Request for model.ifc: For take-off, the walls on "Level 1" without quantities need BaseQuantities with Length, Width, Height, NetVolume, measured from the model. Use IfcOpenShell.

First a look at what the model holds.

```python
import ifcopenshell
import ifcopenshell.util.element
import ifcopenshell.util.unit

model = ifcopenshell.open("model.ifc")
print(model.schema)
for unit_type in ("LENGTHUNIT", "AREAUNIT", "VOLUMEUNIT"):
    print(unit_type, ifcopenshell.util.unit.calculate_unit_scale(model, unit_type))
storey = next(s for s in model.by_type("IfcBuildingStorey") if s.Name == "Level 1")
walls = [e for e in ifcopenshell.util.element.get_decomposition(storey) if e.is_a("IfcWall")]
for e in sorted(walls, key=lambda e: e.id()):
    print(e.id(), e.is_a(), e.Name, list(ifcopenshell.util.element.get_psets(e, qtos_only=True)), sep=" | ")
```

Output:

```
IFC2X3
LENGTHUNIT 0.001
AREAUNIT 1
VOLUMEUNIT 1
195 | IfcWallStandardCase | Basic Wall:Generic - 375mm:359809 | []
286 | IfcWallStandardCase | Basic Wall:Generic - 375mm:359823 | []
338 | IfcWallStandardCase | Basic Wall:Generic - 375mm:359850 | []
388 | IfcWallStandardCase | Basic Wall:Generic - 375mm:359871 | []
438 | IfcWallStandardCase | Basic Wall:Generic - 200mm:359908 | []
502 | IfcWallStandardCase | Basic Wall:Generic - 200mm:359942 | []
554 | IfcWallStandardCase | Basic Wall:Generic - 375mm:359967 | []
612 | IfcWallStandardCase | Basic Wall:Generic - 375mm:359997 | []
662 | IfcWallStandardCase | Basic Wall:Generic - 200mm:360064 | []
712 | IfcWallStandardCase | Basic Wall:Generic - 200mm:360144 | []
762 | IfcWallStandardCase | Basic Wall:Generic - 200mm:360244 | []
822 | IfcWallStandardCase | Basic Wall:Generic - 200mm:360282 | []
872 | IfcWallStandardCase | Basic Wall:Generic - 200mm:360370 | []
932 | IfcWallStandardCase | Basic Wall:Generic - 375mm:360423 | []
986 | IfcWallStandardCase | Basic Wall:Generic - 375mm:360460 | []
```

```python
import ifcopenshell
import ifcopenshell.api.pset
import ifcopenshell.geom
import ifcopenshell.util.element
import ifcopenshell.util.shape
import ifcopenshell.util.unit

model = ifcopenshell.open("model.ifc")
unit_scale = ifcopenshell.util.unit.calculate_unit_scale(model)
volume_scale = ifcopenshell.util.unit.calculate_unit_scale(model, "VOLUMEUNIT")
settings = ifcopenshell.geom.settings()

storey = next(s for s in model.by_type("IfcBuildingStorey") if s.Name == "Level 1")
walls = [e for e in ifcopenshell.util.element.get_decomposition(storey) if e.is_a("IfcWall")]

for e in sorted(walls, key=lambda e: e.id()):
    if ifcopenshell.util.element.get_psets(e, qtos_only=True, should_inherit=False):
        continue
    # Geometry comes back in metres, in the element's own axes.
    shape = ifcopenshell.geom.create_shape(settings, e)
    values = {
        "Length": ifcopenshell.util.shape.get_x(shape.geometry) / unit_scale,
        "Width": ifcopenshell.util.shape.get_y(shape.geometry) / unit_scale,
        "Height": ifcopenshell.util.shape.get_z(shape.geometry) / unit_scale,
        "NetVolume": ifcopenshell.util.shape.get_volume(shape.geometry) / volume_scale,
    }
    qto = ifcopenshell.api.pset.add_qto(model, product=e, name="BaseQuantities")
    ifcopenshell.api.pset.edit_qto(model, qto=qto, properties=values)
    print(e.id(), {k: round(v, 3) for k, v in values.items()})

model.write("model_rev.ifc")
```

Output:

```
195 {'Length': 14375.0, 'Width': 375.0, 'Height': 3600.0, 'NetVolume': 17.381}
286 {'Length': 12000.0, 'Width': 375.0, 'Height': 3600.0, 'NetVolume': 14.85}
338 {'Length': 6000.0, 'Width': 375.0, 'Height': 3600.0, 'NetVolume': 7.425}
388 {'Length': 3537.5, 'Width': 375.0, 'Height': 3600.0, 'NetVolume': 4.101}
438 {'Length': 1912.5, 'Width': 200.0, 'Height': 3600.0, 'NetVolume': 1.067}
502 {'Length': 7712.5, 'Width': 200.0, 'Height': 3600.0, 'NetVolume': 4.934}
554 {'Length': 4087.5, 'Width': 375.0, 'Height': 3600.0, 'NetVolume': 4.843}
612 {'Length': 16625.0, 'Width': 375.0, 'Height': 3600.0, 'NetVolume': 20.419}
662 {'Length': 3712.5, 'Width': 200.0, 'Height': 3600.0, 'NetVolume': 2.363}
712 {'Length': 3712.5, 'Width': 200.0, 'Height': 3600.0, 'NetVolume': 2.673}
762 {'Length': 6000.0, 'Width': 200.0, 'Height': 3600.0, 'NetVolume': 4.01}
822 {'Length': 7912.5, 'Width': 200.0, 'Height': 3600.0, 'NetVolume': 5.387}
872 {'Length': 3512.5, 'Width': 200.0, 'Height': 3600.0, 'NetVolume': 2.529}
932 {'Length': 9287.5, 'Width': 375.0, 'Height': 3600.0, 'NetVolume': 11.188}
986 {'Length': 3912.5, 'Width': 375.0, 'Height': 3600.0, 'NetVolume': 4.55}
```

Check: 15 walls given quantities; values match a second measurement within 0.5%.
